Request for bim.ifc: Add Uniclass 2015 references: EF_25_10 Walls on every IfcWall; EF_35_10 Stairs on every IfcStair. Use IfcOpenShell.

First a look at what the model holds.

```python
import ifcopenshell

model = ifcopenshell.open("bim.ifc")
print(model.schema)
print("classifications:", [c.Name for c in model.by_type("IfcClassification")])
for ifc_class in ("IfcDoor", "IfcRoof", "IfcStair", "IfcWall", "IfcWindow"):
    print(ifc_class, len(model.by_type(ifc_class)))
```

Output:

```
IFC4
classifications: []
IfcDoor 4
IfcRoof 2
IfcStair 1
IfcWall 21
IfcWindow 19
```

```python
import ifcopenshell
import ifcopenshell.api.classification

model = ifcopenshell.open("bim.ifc")

system = ifcopenshell.api.classification.add_classification(model, classification="Uniclass 2015")

codes = {
    "IfcWall": ("EF_25_10", "Walls"),
    "IfcStair": ("EF_35_10", "Stairs"),
}
for ifc_class, (code, name) in codes.items():
    products = model.by_type(ifc_class)
    ifcopenshell.api.classification.add_reference(
        model, products=products, classification=system, identification=code, name=name
    )
    print(code, len(products))

model.write("bim_updated.ifc")
```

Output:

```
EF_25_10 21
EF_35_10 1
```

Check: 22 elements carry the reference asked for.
